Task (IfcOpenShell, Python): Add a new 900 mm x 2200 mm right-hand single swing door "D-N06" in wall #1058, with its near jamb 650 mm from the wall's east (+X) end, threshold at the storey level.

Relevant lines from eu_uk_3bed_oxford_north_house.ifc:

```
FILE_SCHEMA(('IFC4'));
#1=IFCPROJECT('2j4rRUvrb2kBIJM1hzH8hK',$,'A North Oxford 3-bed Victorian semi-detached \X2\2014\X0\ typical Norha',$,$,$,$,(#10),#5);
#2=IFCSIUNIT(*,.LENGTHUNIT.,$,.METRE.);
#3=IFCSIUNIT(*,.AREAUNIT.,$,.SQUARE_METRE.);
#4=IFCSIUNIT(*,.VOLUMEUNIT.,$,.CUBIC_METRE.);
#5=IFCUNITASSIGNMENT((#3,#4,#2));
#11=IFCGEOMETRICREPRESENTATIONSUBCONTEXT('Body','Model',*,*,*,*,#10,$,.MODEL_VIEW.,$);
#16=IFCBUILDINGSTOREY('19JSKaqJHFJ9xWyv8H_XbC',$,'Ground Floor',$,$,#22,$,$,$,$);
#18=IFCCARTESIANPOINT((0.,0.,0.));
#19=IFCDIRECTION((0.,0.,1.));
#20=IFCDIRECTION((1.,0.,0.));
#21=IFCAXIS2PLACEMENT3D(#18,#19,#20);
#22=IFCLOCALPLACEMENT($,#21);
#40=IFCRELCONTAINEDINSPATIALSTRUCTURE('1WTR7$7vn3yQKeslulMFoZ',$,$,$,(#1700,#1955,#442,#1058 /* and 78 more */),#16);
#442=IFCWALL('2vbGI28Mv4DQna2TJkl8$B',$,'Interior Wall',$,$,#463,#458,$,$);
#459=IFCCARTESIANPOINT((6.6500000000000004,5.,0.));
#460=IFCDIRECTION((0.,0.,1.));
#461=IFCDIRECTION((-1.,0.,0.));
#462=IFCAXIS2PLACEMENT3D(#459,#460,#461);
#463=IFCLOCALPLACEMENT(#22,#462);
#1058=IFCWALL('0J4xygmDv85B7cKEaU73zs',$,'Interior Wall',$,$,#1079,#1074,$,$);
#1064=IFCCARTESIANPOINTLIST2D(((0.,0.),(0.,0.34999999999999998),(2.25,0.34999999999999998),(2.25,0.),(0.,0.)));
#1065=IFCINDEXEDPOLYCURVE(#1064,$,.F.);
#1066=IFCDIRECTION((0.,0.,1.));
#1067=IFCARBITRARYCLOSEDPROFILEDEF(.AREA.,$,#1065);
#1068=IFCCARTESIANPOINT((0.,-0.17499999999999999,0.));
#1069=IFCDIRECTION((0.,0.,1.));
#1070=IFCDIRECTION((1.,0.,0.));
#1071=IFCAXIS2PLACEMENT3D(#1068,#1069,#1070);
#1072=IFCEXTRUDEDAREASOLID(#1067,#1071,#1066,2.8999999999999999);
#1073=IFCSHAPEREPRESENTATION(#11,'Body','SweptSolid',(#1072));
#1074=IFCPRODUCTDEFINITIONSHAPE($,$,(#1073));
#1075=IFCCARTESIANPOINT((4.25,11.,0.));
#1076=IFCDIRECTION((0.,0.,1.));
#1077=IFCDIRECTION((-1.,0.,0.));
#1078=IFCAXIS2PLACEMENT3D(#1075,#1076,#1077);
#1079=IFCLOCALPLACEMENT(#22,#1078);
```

```python
import numpy as np
import ifcopenshell
import ifcopenshell.api.feature
import ifcopenshell.api.geometry
import ifcopenshell.api.root
import ifcopenshell.api.spatial
import ifcopenshell.geom
import ifcopenshell.util.element
import ifcopenshell.util.placement
import ifcopenshell.util.representation
import ifcopenshell.util.shape
import ifcopenshell.util.unit

model = ifcopenshell.open("eu_uk_3bed_oxford_north_house.ifc")
unit_scale = ifcopenshell.util.unit.calculate_unit_scale(model)
settings = ifcopenshell.geom.settings()


def volume(element):
    """Net volume in cubic metres, openings subtracted."""
    shape = ifcopenshell.geom.create_shape(settings, element)
    return ifcopenshell.util.shape.get_volume(shape.geometry)


wall = model.by_id(1058)
storey = ifcopenshell.util.element.get_container(wall, ifc_class="IfcBuildingStorey")
context = ifcopenshell.util.representation.get_context(model, "Model", "Body", "MODEL_VIEW")
before = volume(wall)

width, height, from_end, sill = 0.9, 2.2, 0.65, 0.0  # metres

# The wall runs along its own X axis, and the end named is its -X end.
wall_shape = ifcopenshell.geom.create_shape(settings, wall)
x, y, z = ifcopenshell.util.shape.get_vertices(wall_shape.geometry).T
start = x.min() + from_end
face, thickness = float(y.min()), float(y.max() - y.min())
wall_matrix = ifcopenshell.util.placement.get_local_placement(wall.ObjectPlacement)
level = ifcopenshell.util.placement.get_local_placement(storey.ObjectPlacement)[2, 3]


def in_wall(x, y):
    """Placement at x, y metres in the wall's axes, at sill height."""
    matrix = wall_matrix.copy()
    matrix[:, 3] = wall_matrix @ np.array([x / unit_scale, y / unit_scale, 0.0, 1.0])
    matrix[2, 3] = level + sill / unit_scale
    return matrix


# Opening: a box that overshoots both wall faces by 50 mm.
opening = ifcopenshell.api.root.create_entity(model, ifc_class="IfcOpeningElement", predefined_type="OPENING")
box = ifcopenshell.api.geometry.add_wall_representation(
    model, context=context, length=width, height=height, thickness=thickness + 0.1
)
ifcopenshell.api.geometry.assign_representation(model, product=opening, representation=box)
ifcopenshell.api.geometry.edit_object_placement(model, product=opening, matrix=in_wall(start, face - 0.05), is_si=False)
ifcopenshell.api.feature.add_feature(model, feature=opening, element=wall)

door = ifcopenshell.api.root.create_entity(model, ifc_class="IfcDoor", name="D-N06", predefined_type="DOOR")
door.OverallWidth, door.OverallHeight = width / unit_scale, height / unit_scale
door.OperationType = "SINGLE_SWING_RIGHT"
body = ifcopenshell.api.geometry.add_door_representation(
    model,
    context=context,
    overall_width=door.OverallWidth,
    overall_height=door.OverallHeight,
    operation_type="SINGLE_SWING_RIGHT",
    lining_properties={"LiningDepth": thickness / unit_scale, "ThresholdDepth": thickness / unit_scale},
)
ifcopenshell.api.geometry.assign_representation(model, product=door, representation=body)
ifcopenshell.api.spatial.assign_container(model, products=[door], relating_structure=storey)
ifcopenshell.api.feature.add_filling(model, opening=opening, element=door)

# The lining spans the wall, so the door starts at the wall face.
ifcopenshell.api.geometry.edit_object_placement(model, product=door, matrix=in_wall(start, face), is_si=False)

after = volume(wall)

print(f"wall volume {before:.3f} -> {after:.3f} m3")

model.write("eu_uk_3bed_oxford_north_house_edited.ifc")
```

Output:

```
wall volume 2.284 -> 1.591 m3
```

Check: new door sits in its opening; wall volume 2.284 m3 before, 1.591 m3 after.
